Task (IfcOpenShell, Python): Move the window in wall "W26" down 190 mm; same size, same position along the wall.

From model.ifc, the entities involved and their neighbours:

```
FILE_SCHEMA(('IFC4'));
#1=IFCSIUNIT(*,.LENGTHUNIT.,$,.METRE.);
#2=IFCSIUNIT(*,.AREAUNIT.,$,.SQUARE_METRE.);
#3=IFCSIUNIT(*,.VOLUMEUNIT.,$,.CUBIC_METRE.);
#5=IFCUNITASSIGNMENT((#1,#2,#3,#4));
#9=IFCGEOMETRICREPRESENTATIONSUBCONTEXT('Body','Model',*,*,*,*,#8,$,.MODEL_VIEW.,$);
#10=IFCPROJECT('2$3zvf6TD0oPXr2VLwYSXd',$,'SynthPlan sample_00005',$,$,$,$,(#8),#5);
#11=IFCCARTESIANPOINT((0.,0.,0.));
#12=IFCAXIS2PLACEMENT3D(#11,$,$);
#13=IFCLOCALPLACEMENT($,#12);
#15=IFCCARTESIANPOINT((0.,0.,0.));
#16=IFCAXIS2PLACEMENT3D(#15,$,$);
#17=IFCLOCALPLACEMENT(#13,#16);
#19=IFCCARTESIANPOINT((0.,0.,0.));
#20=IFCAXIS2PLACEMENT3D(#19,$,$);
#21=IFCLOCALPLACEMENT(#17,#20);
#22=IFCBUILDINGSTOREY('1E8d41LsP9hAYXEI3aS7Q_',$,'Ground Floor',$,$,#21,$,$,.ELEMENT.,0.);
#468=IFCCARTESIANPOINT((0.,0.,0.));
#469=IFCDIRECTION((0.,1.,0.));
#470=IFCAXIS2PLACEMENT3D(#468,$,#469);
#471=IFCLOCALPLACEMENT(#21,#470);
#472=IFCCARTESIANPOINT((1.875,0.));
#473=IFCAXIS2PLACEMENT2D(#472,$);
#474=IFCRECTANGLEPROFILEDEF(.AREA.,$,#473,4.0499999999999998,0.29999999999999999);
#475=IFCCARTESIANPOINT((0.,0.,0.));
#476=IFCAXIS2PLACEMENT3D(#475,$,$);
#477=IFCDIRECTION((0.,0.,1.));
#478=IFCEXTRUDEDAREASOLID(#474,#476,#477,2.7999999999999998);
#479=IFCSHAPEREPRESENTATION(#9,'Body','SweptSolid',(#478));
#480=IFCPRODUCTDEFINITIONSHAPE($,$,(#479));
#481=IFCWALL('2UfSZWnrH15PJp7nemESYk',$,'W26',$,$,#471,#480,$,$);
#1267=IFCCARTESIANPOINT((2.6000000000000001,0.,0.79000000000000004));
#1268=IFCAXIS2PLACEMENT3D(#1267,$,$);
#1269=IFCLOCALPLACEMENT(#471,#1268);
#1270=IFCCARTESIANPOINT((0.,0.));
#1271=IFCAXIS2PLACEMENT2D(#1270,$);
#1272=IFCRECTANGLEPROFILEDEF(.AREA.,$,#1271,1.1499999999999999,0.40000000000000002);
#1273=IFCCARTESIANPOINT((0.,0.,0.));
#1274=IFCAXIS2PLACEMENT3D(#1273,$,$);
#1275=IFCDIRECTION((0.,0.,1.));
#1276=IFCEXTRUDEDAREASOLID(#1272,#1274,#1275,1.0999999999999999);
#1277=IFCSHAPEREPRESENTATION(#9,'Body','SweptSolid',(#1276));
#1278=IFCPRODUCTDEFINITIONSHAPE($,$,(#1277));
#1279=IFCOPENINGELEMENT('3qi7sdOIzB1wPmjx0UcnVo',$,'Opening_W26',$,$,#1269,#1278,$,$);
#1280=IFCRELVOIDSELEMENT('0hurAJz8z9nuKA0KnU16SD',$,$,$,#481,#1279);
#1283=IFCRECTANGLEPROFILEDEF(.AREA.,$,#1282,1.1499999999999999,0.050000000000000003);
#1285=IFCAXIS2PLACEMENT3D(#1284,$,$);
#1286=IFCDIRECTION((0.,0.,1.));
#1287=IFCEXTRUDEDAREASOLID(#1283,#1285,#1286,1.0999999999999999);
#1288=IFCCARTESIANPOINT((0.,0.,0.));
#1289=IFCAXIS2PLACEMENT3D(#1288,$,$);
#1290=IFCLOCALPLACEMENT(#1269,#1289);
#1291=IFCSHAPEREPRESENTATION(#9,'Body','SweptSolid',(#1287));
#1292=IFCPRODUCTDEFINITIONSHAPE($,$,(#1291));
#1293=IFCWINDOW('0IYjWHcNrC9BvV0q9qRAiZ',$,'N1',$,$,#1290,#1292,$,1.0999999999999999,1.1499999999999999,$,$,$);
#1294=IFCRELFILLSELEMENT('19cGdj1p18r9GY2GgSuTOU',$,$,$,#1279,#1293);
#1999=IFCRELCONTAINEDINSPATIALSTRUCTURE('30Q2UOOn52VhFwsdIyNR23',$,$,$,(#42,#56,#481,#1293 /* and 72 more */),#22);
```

```python
import numpy as np
import ifcopenshell
import ifcopenshell.api.geometry
import ifcopenshell.util.placement
import ifcopenshell.util.unit

model = ifcopenshell.open("model.ifc")
unit_scale = ifcopenshell.util.unit.calculate_unit_scale(model)

window = model.by_id(1293)
opening = window.FillsVoids[0].RelatingOpeningElement
dz = -0.19 / unit_scale

shift = np.array([0.0, 0.0, dz])
# The window is placed relative to its opening, so it follows when the opening moves.
matrix = ifcopenshell.util.placement.get_local_placement(opening.ObjectPlacement)
matrix[:3, 3] += shift
ifcopenshell.api.geometry.edit_object_placement(
    model, product=opening, matrix=matrix, is_si=False, should_transform_children=True
)

print(f"moved by {dz * unit_scale:+.3f} m")

model.write("model_rev.ifc")
```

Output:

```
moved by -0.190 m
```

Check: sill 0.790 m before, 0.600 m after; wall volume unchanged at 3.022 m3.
